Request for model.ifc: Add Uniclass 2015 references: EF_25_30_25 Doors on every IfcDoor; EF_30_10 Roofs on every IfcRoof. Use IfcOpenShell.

First a look at what the model holds.

```python
import ifcopenshell

model = ifcopenshell.open("model.ifc")
print(model.schema)
print("classifications:", [c.Name for c in model.by_type("IfcClassification")])
for ifc_class in ("IfcDoor", "IfcRoof", "IfcStair", "IfcWall", "IfcWindow"):
    print(ifc_class, len(model.by_type(ifc_class)))
```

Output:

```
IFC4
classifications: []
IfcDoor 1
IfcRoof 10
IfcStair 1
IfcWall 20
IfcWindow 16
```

```python
import ifcopenshell
import ifcopenshell.api.classification

model = ifcopenshell.open("model.ifc")

system = ifcopenshell.api.classification.add_classification(model, classification="Uniclass 2015")

codes = {
    "IfcDoor": ("EF_25_30_25", "Doors"),
    "IfcRoof": ("EF_30_10", "Roofs"),
}
for ifc_class, (code, name) in codes.items():
    products = model.by_type(ifc_class)
    ifcopenshell.api.classification.add_reference(
        model, products=products, classification=system, identification=code, name=name
    )
    print(code, len(products))

model.write("model-out.ifc")
```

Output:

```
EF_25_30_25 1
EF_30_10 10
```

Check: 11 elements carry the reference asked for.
